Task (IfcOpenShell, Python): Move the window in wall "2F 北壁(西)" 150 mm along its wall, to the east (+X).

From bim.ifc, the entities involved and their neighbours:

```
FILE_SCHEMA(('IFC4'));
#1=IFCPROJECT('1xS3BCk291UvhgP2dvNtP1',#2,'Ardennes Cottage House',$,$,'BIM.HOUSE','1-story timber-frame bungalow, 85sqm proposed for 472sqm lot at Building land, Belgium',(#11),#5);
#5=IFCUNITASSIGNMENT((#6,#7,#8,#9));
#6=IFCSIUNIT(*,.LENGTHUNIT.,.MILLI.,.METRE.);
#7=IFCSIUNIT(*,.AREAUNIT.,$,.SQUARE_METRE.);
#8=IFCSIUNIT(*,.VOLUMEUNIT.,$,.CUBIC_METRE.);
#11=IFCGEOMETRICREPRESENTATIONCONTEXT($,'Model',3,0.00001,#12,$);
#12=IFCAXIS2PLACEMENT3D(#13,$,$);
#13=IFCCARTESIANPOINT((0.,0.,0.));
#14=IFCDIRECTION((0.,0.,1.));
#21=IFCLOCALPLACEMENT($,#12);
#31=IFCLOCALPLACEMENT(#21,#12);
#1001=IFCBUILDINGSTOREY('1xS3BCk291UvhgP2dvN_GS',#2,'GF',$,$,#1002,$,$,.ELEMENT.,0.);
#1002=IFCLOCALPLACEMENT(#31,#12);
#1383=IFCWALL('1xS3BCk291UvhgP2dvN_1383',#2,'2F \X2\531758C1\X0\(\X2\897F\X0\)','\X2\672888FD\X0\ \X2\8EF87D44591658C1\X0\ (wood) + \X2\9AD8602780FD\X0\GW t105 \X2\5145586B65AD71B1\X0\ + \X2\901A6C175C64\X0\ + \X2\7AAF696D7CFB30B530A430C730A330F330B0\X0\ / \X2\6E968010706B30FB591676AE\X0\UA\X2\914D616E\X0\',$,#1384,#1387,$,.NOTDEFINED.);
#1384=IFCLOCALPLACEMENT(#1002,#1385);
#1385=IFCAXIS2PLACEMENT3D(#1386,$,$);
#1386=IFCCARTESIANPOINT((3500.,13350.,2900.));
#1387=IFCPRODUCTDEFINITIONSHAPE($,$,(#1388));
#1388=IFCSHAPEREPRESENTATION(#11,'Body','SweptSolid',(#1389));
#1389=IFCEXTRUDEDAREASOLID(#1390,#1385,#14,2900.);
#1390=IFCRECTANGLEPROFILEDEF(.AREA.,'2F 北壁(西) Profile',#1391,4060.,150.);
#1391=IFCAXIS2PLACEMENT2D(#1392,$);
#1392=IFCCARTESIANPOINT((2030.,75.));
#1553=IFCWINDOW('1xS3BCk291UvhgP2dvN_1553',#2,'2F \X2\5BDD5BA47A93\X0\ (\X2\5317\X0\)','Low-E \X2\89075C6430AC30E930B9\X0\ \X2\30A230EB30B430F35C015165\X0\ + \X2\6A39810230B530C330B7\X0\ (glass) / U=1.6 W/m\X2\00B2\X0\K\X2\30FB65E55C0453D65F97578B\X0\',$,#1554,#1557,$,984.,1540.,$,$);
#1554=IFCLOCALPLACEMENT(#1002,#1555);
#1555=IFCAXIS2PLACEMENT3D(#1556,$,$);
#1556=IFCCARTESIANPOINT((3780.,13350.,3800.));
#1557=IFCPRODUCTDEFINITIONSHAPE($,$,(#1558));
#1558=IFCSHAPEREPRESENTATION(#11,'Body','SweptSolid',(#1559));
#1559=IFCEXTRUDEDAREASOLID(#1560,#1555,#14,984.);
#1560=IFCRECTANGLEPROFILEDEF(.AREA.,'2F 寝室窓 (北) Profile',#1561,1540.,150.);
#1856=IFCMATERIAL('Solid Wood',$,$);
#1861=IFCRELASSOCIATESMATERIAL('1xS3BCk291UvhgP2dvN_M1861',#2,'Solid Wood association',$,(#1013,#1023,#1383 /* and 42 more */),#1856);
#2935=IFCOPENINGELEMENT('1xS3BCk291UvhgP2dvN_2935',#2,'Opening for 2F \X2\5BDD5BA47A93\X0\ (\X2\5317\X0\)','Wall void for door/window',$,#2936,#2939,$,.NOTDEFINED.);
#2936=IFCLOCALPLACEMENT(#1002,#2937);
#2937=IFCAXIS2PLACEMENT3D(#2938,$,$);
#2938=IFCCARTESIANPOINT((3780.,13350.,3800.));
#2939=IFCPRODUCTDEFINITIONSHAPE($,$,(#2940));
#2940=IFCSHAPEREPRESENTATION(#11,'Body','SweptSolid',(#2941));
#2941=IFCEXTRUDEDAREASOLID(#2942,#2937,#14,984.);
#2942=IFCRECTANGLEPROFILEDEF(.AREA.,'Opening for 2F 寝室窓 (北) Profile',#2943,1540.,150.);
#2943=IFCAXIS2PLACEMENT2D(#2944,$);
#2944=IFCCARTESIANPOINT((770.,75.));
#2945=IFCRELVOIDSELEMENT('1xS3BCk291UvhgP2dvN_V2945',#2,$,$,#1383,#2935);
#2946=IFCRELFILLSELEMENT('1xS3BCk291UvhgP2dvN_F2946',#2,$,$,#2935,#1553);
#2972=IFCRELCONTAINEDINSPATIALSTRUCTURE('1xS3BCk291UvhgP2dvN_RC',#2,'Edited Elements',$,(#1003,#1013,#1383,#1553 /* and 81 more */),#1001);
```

```python
import ifcopenshell
import ifcopenshell.api.geometry
import ifcopenshell.util.placement
import ifcopenshell.util.unit

model = ifcopenshell.open("bim.ifc")
unit_scale = ifcopenshell.util.unit.calculate_unit_scale(model)

window = model.by_id(1553)
opening = window.FillsVoids[0].RelatingOpeningElement
wall = opening.VoidsElements[0].RelatingBuildingElement

wall_matrix = ifcopenshell.util.placement.get_local_placement(wall.ObjectPlacement)
shift = wall_matrix[:3, 0] * 0.15 / unit_scale
before = ifcopenshell.util.placement.get_local_placement(window.ObjectPlacement)[:3, 3].copy()

# The window is not placed relative to its opening, so move both.
for product in (opening, window):
    matrix = ifcopenshell.util.placement.get_local_placement(product.ObjectPlacement)
    matrix[:3, 3] += shift
    ifcopenshell.api.geometry.edit_object_placement(model, product=product, matrix=matrix, is_si=False)

after = ifcopenshell.util.placement.get_local_placement(window.ObjectPlacement)[:3, 3]
print("window moved by", (after - before).round(3) + 0.0)

model.write("bim-out.ifc")
```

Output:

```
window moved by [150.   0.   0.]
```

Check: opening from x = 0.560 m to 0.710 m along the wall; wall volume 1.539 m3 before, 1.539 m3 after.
